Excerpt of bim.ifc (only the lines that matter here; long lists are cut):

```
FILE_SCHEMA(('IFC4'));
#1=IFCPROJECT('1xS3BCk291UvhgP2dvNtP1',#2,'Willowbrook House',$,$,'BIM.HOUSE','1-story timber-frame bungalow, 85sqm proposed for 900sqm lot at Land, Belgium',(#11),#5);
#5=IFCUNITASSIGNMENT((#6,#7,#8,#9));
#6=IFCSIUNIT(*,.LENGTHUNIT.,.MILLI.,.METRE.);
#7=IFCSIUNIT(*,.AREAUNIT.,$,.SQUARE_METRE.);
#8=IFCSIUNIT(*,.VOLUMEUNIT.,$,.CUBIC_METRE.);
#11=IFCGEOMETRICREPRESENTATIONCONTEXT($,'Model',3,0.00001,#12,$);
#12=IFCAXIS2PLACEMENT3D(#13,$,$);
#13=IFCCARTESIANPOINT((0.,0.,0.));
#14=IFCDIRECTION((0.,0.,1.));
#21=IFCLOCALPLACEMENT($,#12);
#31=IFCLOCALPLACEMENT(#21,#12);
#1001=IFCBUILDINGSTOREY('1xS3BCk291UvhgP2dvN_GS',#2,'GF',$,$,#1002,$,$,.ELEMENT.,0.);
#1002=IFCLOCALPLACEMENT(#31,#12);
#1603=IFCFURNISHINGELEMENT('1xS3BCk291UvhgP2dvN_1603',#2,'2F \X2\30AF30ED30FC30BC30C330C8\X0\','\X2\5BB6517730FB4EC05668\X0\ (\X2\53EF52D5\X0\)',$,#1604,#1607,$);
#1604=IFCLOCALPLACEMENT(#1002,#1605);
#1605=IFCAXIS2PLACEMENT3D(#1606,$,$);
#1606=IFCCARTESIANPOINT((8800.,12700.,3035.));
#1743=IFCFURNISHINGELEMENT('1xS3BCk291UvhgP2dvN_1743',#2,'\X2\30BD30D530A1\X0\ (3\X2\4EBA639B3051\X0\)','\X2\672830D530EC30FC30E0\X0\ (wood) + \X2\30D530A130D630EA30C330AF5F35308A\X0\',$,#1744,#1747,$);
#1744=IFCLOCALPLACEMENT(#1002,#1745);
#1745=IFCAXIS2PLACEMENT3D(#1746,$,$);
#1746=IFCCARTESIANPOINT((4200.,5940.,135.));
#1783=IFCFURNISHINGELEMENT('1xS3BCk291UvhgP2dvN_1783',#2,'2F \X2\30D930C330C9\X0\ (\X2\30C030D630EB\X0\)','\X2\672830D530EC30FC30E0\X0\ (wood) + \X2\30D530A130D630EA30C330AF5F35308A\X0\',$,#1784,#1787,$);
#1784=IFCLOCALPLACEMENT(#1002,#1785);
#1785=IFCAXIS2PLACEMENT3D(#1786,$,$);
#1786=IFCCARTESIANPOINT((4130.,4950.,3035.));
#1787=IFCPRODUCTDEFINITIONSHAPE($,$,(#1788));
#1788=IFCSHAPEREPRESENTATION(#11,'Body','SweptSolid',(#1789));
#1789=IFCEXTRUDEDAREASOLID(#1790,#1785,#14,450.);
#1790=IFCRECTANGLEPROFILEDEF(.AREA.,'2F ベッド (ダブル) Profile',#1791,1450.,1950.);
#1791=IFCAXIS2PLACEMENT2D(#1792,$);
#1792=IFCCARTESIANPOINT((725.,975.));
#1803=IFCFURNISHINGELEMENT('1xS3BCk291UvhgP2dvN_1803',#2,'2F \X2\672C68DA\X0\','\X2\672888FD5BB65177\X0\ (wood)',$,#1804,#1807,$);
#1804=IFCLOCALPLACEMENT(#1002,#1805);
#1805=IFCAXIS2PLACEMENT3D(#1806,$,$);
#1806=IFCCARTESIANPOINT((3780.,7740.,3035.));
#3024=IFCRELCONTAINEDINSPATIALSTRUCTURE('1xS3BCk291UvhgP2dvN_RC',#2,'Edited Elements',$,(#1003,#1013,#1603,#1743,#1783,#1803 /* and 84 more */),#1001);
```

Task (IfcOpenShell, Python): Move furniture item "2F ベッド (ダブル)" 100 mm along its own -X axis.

```python
import ifcopenshell
import ifcopenshell.api.geometry
import ifcopenshell.util.placement

model = ifcopenshell.open("bim.ifc")

item = model.by_guid("1xS3BCk291UvhgP2dvN_1783")
matrix = ifcopenshell.util.placement.get_local_placement(item.ObjectPlacement)
matrix[:3, 3] -= matrix[:3, 0] * 100.0
ifcopenshell.api.geometry.edit_object_placement(model, product=item, matrix=matrix, is_si=False)

print(ifcopenshell.util.placement.get_local_placement(item.ObjectPlacement).round(3) + 0.0)

model.write("bim_v2.ifc")
```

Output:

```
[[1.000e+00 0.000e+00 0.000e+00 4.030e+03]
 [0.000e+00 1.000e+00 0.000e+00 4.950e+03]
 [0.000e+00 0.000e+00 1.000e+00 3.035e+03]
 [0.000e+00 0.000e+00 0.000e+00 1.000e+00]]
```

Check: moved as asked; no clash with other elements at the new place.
